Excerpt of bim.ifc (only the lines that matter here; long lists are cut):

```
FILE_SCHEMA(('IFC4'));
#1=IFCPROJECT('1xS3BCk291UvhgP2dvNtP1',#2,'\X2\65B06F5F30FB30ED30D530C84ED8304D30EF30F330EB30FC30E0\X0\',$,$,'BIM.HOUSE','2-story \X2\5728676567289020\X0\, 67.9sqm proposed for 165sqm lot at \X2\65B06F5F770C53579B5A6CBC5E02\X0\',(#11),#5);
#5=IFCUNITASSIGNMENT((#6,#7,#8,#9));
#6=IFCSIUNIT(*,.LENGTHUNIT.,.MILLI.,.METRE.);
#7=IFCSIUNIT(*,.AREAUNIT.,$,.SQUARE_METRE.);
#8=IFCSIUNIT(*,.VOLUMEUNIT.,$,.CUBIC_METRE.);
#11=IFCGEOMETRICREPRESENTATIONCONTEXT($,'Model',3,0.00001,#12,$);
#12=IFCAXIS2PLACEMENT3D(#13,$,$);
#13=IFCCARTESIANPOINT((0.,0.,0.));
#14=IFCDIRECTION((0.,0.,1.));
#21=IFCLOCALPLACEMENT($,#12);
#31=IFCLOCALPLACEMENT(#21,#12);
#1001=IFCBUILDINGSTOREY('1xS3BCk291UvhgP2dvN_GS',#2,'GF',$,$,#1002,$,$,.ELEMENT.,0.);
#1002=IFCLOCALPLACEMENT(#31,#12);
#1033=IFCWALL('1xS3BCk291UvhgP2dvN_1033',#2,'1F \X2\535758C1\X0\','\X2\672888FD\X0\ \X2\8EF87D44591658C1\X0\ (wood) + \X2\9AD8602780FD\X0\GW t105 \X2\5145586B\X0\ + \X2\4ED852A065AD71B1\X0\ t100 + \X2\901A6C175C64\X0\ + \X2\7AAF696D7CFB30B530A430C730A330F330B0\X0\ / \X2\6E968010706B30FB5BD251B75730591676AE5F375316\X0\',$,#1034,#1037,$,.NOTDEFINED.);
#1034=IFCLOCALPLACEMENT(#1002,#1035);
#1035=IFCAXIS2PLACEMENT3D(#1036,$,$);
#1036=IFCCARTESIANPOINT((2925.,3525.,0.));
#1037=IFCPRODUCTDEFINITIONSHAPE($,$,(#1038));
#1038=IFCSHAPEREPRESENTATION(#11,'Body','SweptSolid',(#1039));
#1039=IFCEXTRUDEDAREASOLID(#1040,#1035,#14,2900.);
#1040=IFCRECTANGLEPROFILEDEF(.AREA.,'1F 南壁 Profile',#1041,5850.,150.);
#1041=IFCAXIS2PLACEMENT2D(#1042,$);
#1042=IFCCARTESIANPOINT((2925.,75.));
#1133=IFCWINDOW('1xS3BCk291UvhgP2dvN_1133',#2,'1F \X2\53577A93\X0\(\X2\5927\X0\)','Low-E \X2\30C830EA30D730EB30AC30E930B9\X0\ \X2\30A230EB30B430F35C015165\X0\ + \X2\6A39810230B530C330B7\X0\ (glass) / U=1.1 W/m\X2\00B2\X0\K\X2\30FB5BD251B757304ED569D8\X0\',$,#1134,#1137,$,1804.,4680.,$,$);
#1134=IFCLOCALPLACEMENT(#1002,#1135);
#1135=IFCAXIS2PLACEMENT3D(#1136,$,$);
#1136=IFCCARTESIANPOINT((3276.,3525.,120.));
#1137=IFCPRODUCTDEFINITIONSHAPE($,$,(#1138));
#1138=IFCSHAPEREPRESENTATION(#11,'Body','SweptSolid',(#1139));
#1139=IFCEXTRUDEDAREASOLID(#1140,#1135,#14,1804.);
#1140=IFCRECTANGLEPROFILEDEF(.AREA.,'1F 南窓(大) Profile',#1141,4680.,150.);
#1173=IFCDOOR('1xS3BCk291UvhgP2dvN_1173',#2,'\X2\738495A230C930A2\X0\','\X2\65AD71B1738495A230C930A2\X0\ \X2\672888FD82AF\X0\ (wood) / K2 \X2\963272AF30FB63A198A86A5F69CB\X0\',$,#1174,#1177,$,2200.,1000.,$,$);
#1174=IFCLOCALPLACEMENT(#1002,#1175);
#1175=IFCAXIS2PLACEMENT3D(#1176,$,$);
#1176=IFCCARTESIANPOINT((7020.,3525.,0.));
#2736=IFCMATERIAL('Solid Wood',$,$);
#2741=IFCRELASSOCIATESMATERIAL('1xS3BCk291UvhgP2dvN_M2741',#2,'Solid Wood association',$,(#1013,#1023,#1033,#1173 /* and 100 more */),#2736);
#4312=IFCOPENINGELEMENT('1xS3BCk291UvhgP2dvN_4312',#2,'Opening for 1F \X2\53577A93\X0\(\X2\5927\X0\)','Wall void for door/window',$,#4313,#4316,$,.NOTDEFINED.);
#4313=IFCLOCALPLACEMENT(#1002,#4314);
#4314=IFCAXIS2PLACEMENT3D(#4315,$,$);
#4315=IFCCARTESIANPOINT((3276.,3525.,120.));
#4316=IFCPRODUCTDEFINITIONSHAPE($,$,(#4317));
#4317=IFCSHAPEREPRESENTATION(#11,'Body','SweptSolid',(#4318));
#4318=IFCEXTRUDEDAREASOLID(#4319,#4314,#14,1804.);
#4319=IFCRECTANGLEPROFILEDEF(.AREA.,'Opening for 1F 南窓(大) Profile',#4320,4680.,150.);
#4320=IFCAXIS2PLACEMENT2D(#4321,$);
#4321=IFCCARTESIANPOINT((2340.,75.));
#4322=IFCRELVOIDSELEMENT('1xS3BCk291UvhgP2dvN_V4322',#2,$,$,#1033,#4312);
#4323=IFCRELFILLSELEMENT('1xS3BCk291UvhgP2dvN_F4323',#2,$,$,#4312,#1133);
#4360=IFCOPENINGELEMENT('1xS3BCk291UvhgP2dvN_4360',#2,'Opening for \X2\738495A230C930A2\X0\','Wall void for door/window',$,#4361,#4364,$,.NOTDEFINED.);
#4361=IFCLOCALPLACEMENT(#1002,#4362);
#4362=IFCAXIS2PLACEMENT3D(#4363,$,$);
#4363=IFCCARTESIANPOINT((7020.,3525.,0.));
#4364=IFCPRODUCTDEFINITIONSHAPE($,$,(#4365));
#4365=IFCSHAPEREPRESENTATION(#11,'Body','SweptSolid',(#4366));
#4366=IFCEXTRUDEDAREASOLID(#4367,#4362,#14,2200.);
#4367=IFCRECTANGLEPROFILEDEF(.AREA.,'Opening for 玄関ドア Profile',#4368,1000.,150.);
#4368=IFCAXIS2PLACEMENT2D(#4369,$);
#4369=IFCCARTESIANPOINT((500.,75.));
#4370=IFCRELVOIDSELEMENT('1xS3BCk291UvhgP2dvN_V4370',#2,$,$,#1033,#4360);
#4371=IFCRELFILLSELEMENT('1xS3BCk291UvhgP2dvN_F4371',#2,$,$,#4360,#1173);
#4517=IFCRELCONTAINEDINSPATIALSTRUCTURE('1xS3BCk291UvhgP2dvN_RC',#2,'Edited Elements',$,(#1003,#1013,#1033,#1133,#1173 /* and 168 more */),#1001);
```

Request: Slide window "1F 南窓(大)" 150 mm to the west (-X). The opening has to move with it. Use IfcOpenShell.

```python
import ifcopenshell
import ifcopenshell.api.geometry
import ifcopenshell.util.placement

model = ifcopenshell.open("bim.ifc")

window = model.by_guid("1xS3BCk291UvhgP2dvN_1133")
opening = window.FillsVoids[0].RelatingOpeningElement
wall = opening.VoidsElements[0].RelatingBuildingElement

wall_matrix = ifcopenshell.util.placement.get_local_placement(wall.ObjectPlacement)
shift = wall_matrix[:3, 0] * -150.0
before = ifcopenshell.util.placement.get_local_placement(window.ObjectPlacement)[:3, 3].copy()

# The window is not placed relative to its opening, so move both.
for product in (opening, window):
    matrix = ifcopenshell.util.placement.get_local_placement(product.ObjectPlacement)
    matrix[:3, 3] += shift
    ifcopenshell.api.geometry.edit_object_placement(model, product=product, matrix=matrix, is_si=False)

after = ifcopenshell.util.placement.get_local_placement(window.ObjectPlacement)[:3, 3]
print("window moved by", (after - before).round(3) + 0.0)

model.write("bim-out.ifc")
```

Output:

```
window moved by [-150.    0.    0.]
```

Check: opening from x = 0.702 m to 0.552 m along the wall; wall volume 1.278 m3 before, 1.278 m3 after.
